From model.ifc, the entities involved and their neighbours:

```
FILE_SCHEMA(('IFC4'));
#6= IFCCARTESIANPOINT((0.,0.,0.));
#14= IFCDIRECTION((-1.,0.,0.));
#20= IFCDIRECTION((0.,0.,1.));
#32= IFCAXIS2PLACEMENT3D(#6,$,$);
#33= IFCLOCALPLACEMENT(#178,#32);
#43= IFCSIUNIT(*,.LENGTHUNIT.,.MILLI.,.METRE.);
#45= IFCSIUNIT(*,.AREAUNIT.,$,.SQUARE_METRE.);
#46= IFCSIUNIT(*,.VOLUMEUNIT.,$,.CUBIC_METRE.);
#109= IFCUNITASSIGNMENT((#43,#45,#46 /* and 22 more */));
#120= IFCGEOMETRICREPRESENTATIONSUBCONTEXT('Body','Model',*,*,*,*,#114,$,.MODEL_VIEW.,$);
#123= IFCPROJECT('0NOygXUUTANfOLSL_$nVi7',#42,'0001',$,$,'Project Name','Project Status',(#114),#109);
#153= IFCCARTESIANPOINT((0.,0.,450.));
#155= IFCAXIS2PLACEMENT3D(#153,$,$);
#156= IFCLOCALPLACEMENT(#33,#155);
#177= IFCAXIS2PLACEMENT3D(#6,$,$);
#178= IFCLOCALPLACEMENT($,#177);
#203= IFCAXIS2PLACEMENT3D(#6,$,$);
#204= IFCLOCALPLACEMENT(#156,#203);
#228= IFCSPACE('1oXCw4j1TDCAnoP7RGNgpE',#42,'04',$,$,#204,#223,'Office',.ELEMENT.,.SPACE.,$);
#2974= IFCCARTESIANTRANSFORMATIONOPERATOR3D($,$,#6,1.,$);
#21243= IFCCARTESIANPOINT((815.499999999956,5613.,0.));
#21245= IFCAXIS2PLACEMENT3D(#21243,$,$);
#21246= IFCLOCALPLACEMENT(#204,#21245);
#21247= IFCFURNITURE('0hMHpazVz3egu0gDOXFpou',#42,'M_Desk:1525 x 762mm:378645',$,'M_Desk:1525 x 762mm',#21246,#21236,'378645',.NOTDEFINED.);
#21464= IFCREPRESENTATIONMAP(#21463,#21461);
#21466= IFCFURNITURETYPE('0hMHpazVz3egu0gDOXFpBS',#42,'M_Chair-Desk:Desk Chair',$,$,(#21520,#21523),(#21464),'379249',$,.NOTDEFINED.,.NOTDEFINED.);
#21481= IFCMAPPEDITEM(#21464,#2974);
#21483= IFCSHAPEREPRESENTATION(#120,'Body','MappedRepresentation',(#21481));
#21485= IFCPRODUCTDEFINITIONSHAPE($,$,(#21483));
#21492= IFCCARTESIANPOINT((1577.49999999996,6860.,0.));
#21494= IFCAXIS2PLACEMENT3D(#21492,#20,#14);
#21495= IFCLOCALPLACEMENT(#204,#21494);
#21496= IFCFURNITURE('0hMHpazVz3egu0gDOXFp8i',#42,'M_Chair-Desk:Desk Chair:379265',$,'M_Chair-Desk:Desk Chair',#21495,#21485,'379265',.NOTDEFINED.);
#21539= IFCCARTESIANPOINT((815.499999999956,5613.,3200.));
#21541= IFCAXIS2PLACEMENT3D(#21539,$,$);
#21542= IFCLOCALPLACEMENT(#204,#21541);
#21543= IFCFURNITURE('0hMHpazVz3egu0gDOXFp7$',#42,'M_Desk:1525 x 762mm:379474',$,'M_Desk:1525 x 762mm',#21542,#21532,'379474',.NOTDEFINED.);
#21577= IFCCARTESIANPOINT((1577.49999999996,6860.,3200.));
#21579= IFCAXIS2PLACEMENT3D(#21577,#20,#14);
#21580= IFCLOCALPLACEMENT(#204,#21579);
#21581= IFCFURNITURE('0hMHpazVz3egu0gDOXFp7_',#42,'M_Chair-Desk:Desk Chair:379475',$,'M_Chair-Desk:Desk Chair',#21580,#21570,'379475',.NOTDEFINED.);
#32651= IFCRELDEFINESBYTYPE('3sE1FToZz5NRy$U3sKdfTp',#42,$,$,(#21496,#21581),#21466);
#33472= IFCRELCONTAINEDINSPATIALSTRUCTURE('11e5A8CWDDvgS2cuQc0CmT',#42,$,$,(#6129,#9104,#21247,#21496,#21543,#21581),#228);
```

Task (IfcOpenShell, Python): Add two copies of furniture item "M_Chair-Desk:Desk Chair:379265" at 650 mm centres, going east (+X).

```python
import numpy as np
import ifcopenshell
import ifcopenshell.api.geometry
import ifcopenshell.api.root
import ifcopenshell.util.element
import ifcopenshell.util.placement
import ifcopenshell.util.unit

model = ifcopenshell.open("model.ifc")
unit_scale = ifcopenshell.util.unit.calculate_unit_scale(model)


def reuse_history(source, copy):
    """copy_class also copies each property set's owner history, people and application; keep the originals."""
    for rel in copy.IsDefinedBy:
        if rel.is_a("IfcRelDefinesByProperties") and (history := rel.RelatingPropertyDefinition.OwnerHistory):
            rel.RelatingPropertyDefinition.OwnerHistory = source.OwnerHistory
            ifcopenshell.util.element.remove_deep2(model, history)


source = model.by_guid("0hMHpazVz3egu0gDOXFp8i")
base = ifcopenshell.util.placement.get_local_placement(source.ObjectPlacement)
step = np.array([1.0, 0.0, 0.0]) * 0.65 / unit_scale

for i in range(1, 3):
    copy = ifcopenshell.api.root.copy_class(model, product=source)
    copy.Representation = ifcopenshell.util.element.copy_deep(
        model, source.Representation, exclude=["IfcGeometricRepresentationContext", "IfcRepresentationMap"]
    )
    copy.Name = "M_Chair-Desk:Desk Chair"
    copy.Tag = None
    reuse_history(source, copy)
    matrix = base.copy()
    matrix[:3, 3] += i * step
    print("added at", matrix[:3, 3].round(3) + 0.0)
    ifcopenshell.api.geometry.edit_object_placement(model, product=copy, matrix=matrix, is_si=False)

model.write("model_rev.ifc")
```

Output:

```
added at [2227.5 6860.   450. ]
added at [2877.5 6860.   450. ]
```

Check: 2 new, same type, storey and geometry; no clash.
